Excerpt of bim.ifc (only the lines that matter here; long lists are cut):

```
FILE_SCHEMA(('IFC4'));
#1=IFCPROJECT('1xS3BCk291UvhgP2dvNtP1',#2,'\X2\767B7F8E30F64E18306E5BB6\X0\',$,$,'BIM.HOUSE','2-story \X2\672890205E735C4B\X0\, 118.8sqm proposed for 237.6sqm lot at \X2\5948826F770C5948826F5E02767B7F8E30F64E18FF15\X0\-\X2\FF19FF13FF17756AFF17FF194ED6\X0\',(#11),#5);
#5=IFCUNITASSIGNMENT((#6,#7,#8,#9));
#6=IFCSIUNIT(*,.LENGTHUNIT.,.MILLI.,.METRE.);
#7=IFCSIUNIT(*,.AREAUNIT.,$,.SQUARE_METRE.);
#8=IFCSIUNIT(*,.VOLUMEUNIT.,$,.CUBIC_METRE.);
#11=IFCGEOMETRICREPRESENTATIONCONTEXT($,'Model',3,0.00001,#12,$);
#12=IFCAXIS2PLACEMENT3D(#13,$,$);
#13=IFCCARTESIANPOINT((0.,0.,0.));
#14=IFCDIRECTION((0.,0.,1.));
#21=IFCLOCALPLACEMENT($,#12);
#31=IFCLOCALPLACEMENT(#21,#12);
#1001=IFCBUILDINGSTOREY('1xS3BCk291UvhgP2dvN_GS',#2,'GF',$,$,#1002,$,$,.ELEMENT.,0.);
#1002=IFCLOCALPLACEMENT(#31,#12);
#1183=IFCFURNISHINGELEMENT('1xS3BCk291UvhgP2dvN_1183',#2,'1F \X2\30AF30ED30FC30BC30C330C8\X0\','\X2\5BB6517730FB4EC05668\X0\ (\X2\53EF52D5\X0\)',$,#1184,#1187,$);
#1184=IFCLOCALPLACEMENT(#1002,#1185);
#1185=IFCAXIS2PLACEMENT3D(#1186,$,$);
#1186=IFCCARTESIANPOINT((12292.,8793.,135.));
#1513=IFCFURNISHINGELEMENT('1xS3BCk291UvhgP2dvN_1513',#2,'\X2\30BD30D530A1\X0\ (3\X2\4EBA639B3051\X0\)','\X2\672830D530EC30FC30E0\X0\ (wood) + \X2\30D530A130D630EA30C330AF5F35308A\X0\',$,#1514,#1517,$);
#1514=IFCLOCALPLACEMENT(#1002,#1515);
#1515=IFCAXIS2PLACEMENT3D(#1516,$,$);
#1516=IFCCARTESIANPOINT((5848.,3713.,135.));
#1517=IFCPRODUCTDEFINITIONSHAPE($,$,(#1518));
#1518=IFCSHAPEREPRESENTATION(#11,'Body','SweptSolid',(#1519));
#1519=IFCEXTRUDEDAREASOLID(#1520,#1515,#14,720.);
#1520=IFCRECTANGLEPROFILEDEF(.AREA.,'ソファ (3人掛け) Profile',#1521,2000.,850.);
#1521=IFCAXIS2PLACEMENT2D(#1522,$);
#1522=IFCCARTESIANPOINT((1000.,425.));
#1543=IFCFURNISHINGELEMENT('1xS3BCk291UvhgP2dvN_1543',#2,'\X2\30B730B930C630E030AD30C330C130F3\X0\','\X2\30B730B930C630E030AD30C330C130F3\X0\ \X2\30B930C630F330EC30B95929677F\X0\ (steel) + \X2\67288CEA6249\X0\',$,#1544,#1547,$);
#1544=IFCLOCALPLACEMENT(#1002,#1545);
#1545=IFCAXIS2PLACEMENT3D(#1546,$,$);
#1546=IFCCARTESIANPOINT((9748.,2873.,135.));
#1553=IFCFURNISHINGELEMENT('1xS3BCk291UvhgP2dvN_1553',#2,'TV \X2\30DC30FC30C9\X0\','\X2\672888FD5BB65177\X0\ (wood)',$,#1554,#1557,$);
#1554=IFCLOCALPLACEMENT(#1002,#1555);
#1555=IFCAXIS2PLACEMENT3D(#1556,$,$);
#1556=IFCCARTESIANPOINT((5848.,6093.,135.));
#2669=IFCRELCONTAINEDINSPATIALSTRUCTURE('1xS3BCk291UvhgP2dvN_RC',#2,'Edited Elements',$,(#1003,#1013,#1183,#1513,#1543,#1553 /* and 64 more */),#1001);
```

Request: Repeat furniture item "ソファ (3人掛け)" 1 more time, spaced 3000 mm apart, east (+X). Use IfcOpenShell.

```python
import numpy as np
import ifcopenshell
import ifcopenshell.api.geometry
import ifcopenshell.api.root
import ifcopenshell.util.element
import ifcopenshell.util.placement

model = ifcopenshell.open("bim.ifc")


def reuse_history(source, copy):
    """copy_class also copies each property set's owner history, people and application; keep the originals."""
    for rel in copy.IsDefinedBy:
        if rel.is_a("IfcRelDefinesByProperties") and (history := rel.RelatingPropertyDefinition.OwnerHistory):
            rel.RelatingPropertyDefinition.OwnerHistory = source.OwnerHistory
            ifcopenshell.util.element.remove_deep2(model, history)


source = model.by_guid("1xS3BCk291UvhgP2dvN_1513")
base = ifcopenshell.util.placement.get_local_placement(source.ObjectPlacement)
step = np.array([1.0, 0.0, 0.0]) * 3000.0

for i in range(1, 2):
    copy = ifcopenshell.api.root.copy_class(model, product=source)
    copy.Representation = ifcopenshell.util.element.copy_deep(
        model, source.Representation, exclude=["IfcGeometricRepresentationContext", "IfcRepresentationMap"]
    )
    reuse_history(source, copy)
    matrix = base.copy()
    matrix[:3, 3] += i * step
    print("added at", matrix[:3, 3].round(3) + 0.0)
    ifcopenshell.api.geometry.edit_object_placement(model, product=copy, matrix=matrix, is_si=False)

model.write("bim_edited.ifc")
```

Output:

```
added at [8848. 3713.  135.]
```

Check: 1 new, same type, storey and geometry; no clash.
